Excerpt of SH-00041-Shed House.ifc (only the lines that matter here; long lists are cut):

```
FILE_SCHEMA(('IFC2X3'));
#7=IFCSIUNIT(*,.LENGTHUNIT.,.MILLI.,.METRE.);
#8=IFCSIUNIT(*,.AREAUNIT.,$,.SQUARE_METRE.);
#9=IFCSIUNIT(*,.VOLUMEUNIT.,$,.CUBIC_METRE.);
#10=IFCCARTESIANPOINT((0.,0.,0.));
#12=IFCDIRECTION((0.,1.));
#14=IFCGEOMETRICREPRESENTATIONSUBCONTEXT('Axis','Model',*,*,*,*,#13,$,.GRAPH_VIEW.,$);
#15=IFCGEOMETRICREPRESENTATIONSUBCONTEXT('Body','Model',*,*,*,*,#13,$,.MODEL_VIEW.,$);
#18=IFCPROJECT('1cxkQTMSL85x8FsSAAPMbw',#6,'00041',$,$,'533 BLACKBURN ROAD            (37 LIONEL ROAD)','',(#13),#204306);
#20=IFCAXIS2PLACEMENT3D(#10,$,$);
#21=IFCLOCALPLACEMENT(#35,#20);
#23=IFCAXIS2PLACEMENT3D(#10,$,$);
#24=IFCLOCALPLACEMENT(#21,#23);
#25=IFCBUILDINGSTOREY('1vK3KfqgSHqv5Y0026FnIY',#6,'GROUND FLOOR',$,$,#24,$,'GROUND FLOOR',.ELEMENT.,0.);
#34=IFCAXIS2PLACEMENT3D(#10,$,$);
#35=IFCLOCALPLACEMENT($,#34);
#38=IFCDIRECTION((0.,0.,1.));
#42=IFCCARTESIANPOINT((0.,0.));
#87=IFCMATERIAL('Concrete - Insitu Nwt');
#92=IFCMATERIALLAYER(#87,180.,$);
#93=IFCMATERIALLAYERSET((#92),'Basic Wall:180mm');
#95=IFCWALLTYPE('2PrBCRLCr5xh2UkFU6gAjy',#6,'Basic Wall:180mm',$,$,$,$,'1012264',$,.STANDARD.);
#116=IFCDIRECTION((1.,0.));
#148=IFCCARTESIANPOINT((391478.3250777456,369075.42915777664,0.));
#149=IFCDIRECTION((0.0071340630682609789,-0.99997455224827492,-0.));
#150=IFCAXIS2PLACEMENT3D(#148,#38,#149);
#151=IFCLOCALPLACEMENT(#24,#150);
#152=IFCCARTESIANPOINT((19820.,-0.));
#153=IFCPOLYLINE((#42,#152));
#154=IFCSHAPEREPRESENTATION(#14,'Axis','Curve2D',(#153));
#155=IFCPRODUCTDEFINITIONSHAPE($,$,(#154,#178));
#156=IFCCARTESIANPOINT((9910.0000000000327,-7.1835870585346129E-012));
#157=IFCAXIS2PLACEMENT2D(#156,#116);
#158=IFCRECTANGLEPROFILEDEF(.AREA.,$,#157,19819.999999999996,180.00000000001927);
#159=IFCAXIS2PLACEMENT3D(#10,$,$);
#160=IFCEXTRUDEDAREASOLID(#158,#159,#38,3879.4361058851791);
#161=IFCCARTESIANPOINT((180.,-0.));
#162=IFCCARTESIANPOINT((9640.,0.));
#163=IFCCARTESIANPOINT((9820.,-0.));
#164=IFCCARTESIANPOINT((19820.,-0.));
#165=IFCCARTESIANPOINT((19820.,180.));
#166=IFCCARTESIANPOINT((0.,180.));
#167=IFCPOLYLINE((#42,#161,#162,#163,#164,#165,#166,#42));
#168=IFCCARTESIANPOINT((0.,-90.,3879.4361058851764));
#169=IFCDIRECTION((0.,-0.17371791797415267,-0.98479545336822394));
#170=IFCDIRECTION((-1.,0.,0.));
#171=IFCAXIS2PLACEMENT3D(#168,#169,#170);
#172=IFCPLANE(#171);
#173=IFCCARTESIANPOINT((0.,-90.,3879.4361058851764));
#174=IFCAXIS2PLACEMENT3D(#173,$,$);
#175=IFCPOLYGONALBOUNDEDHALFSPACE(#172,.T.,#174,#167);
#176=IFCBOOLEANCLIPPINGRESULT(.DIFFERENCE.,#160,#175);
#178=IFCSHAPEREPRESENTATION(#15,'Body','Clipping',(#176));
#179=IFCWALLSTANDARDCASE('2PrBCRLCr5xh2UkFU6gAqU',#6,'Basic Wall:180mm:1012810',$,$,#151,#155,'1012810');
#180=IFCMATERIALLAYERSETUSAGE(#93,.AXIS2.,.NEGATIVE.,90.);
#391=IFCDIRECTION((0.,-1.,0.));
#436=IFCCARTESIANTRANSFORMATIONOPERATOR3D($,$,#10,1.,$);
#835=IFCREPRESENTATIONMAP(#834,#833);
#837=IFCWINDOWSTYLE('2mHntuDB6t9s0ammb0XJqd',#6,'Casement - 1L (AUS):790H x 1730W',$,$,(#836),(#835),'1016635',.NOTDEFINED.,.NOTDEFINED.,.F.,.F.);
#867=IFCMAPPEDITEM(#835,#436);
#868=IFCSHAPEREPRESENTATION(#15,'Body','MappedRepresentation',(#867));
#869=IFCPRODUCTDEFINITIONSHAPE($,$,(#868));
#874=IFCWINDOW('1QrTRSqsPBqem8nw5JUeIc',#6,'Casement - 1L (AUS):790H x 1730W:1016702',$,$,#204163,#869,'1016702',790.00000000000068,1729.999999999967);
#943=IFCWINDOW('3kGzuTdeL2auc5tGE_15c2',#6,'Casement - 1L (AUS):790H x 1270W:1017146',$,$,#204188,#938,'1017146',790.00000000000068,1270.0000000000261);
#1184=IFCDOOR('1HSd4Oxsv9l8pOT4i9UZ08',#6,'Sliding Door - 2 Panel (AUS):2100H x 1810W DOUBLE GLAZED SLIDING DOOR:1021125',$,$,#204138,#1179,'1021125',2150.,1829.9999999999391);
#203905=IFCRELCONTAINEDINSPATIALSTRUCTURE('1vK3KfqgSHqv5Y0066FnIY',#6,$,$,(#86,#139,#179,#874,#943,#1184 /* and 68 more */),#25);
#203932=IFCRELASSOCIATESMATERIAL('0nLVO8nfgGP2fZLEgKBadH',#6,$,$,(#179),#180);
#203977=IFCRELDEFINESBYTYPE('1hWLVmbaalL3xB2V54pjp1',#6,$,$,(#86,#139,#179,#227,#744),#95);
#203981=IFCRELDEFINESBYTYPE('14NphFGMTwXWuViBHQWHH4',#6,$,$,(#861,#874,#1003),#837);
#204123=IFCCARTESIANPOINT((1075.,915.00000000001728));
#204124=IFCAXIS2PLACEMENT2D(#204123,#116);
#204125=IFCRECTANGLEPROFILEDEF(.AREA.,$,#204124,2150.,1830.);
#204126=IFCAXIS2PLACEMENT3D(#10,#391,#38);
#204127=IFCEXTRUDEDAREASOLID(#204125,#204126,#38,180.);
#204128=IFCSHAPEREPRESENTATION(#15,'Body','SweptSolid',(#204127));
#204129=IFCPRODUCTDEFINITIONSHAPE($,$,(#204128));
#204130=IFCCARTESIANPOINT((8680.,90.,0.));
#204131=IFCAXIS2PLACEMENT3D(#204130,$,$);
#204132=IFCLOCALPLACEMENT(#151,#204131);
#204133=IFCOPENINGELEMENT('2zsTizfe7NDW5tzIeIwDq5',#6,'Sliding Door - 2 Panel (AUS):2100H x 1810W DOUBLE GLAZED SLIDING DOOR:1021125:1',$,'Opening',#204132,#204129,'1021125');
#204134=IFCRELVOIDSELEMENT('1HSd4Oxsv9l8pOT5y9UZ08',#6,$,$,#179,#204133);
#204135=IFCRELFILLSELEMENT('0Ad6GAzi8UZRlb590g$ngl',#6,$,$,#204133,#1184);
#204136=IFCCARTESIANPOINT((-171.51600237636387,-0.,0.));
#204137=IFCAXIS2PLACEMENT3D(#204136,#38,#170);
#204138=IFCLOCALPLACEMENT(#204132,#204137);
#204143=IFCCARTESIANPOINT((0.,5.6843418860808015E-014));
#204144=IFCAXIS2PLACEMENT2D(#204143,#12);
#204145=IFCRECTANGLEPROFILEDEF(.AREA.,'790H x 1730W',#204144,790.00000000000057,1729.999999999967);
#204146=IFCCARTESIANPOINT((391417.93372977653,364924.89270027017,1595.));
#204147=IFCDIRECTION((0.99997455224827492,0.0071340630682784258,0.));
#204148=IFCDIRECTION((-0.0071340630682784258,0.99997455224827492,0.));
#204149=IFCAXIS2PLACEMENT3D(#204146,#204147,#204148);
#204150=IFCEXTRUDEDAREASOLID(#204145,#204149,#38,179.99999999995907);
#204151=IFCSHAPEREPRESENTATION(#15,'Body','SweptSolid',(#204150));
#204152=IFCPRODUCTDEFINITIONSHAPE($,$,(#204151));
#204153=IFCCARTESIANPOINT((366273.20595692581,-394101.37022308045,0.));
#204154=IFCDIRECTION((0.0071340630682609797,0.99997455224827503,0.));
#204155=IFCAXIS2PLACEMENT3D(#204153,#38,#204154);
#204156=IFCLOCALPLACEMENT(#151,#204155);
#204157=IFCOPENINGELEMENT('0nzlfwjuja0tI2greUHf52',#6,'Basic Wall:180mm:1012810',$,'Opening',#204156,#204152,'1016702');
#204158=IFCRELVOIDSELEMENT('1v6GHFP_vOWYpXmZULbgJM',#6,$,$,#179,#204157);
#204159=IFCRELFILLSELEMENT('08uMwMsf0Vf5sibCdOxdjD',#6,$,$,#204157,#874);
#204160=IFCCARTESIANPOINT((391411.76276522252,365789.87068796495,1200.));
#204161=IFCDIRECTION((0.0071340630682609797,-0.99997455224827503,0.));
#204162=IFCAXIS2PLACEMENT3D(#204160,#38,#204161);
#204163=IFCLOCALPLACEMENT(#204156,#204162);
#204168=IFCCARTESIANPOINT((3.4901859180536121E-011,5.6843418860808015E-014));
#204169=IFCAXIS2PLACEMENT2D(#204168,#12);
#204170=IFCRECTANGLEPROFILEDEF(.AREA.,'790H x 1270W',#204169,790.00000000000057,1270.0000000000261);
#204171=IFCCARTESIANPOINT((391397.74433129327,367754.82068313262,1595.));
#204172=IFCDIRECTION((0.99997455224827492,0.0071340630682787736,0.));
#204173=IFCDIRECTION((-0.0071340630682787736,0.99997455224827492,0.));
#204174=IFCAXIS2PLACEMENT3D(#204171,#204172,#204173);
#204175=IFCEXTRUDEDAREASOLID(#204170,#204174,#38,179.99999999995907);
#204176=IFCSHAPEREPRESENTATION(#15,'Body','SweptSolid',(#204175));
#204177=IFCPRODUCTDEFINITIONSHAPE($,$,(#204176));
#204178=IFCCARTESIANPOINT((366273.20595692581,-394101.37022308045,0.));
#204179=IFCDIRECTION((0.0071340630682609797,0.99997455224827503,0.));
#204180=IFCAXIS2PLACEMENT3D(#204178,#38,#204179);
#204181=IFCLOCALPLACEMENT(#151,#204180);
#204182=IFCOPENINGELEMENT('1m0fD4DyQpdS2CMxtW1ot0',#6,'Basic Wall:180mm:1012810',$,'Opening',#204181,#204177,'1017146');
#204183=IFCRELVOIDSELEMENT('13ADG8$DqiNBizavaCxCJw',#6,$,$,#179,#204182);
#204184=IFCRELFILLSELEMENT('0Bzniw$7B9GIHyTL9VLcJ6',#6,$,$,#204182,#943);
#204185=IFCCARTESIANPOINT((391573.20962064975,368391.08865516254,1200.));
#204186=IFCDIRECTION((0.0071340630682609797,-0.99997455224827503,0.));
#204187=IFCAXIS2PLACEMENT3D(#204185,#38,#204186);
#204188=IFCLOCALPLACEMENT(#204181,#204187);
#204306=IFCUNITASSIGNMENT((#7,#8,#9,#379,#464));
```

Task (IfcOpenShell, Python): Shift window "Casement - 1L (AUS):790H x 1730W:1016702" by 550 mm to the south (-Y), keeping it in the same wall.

```python
import ifcopenshell
import ifcopenshell.api.geometry
import ifcopenshell.util.placement

model = ifcopenshell.open("SH-00041-Shed House.ifc")

window = model.by_guid("1QrTRSqsPBqem8nw5JUeIc")
opening = window.FillsVoids[0].RelatingOpeningElement
wall = opening.VoidsElements[0].RelatingBuildingElement

wall_matrix = ifcopenshell.util.placement.get_local_placement(wall.ObjectPlacement)
shift = wall_matrix[:3, 0] * 550.0
before = ifcopenshell.util.placement.get_local_placement(window.ObjectPlacement)[:3, 3].copy()

# The window is placed relative to its opening, so it follows when the opening moves.
matrix = ifcopenshell.util.placement.get_local_placement(opening.ObjectPlacement)
matrix[:3, 3] += shift
ifcopenshell.api.geometry.edit_object_placement(
    model, product=opening, matrix=matrix, is_si=False, should_transform_children=True
)

after = ifcopenshell.util.placement.get_local_placement(window.ObjectPlacement)[:3, 3]
print("window moved by", (after - before).round(3) + 0.0)

model.write("SH-00041-Shed House_v2.ifc")
```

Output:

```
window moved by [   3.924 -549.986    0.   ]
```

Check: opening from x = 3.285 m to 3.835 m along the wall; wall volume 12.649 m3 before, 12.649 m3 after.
